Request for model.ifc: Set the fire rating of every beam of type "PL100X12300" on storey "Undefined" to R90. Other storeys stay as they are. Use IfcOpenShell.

First a look at what the model holds.

```python
import ifcopenshell
import ifcopenshell.util.element

model = ifcopenshell.open("model.ifc")
print(model.schema)
storey = next(s for s in model.by_type("IfcBuildingStorey") if s.Name == "Undefined")
beams = [e for e in ifcopenshell.util.element.get_decomposition(storey) if e.is_a("IfcBeam")]
seen = {}
for e in beams:
    element_type = ifcopenshell.util.element.get_type(e)
    key = (element_type.Name if element_type != e and element_type else None, ifcopenshell.util.element.get_pset(e, "Pset_BeamCommon", "FireRating"))
    seen[key] = seen.get(key, 0) + 1
for (name, value), count in sorted(seen.items(), key=str):
    print(count, "x", name, "|", value)
```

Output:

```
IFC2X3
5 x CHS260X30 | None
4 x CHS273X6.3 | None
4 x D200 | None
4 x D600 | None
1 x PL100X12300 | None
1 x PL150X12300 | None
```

```python
import ifcopenshell
import ifcopenshell.api.pset
import ifcopenshell.util.element

model = ifcopenshell.open("model.ifc")

storey = next(s for s in model.by_type("IfcBuildingStorey") if s.Name == "Undefined")
beams = [e for e in ifcopenshell.util.element.get_decomposition(storey) if e.is_a("IfcBeam")]

count = 0
for e in beams:
    element_type = ifcopenshell.util.element.get_type(e)
    if element_type in (None, e) or element_type.Name != "PL100X12300":
        continue
    # add_pset returns the element's existing set when there is one.
    pset = ifcopenshell.api.pset.add_pset(model, product=e, name="Pset_BeamCommon")
    ifcopenshell.api.pset.edit_pset(model, pset=pset, properties={"FireRating": "R90"})
    count += 1

print(count, "beams updated")

model.write("model-out.ifc")
```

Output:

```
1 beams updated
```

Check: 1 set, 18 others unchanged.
